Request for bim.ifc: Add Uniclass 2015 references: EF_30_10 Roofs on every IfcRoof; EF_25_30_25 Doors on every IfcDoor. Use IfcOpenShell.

First a look at what the model holds.

```python
import ifcopenshell

model = ifcopenshell.open("bim.ifc")
print(model.schema)
print("classifications:", [c.Name for c in model.by_type("IfcClassification")])
for ifc_class in ("IfcDoor", "IfcRoof", "IfcStair", "IfcWall", "IfcWindow"):
    print(ifc_class, len(model.by_type(ifc_class)))
```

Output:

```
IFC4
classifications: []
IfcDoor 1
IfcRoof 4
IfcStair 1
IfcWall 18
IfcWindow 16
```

```python
import ifcopenshell
import ifcopenshell.api.classification

model = ifcopenshell.open("bim.ifc")

system = ifcopenshell.api.classification.add_classification(model, classification="Uniclass 2015")

codes = {
    "IfcRoof": ("EF_30_10", "Roofs"),
    "IfcDoor": ("EF_25_30_25", "Doors"),
}
for ifc_class, (code, name) in codes.items():
    products = model.by_type(ifc_class)
    ifcopenshell.api.classification.add_reference(
        model, products=products, classification=system, identification=code, name=name
    )
    print(code, len(products))

model.write("bim_v2.ifc")
```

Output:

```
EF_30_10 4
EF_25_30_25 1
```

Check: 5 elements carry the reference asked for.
